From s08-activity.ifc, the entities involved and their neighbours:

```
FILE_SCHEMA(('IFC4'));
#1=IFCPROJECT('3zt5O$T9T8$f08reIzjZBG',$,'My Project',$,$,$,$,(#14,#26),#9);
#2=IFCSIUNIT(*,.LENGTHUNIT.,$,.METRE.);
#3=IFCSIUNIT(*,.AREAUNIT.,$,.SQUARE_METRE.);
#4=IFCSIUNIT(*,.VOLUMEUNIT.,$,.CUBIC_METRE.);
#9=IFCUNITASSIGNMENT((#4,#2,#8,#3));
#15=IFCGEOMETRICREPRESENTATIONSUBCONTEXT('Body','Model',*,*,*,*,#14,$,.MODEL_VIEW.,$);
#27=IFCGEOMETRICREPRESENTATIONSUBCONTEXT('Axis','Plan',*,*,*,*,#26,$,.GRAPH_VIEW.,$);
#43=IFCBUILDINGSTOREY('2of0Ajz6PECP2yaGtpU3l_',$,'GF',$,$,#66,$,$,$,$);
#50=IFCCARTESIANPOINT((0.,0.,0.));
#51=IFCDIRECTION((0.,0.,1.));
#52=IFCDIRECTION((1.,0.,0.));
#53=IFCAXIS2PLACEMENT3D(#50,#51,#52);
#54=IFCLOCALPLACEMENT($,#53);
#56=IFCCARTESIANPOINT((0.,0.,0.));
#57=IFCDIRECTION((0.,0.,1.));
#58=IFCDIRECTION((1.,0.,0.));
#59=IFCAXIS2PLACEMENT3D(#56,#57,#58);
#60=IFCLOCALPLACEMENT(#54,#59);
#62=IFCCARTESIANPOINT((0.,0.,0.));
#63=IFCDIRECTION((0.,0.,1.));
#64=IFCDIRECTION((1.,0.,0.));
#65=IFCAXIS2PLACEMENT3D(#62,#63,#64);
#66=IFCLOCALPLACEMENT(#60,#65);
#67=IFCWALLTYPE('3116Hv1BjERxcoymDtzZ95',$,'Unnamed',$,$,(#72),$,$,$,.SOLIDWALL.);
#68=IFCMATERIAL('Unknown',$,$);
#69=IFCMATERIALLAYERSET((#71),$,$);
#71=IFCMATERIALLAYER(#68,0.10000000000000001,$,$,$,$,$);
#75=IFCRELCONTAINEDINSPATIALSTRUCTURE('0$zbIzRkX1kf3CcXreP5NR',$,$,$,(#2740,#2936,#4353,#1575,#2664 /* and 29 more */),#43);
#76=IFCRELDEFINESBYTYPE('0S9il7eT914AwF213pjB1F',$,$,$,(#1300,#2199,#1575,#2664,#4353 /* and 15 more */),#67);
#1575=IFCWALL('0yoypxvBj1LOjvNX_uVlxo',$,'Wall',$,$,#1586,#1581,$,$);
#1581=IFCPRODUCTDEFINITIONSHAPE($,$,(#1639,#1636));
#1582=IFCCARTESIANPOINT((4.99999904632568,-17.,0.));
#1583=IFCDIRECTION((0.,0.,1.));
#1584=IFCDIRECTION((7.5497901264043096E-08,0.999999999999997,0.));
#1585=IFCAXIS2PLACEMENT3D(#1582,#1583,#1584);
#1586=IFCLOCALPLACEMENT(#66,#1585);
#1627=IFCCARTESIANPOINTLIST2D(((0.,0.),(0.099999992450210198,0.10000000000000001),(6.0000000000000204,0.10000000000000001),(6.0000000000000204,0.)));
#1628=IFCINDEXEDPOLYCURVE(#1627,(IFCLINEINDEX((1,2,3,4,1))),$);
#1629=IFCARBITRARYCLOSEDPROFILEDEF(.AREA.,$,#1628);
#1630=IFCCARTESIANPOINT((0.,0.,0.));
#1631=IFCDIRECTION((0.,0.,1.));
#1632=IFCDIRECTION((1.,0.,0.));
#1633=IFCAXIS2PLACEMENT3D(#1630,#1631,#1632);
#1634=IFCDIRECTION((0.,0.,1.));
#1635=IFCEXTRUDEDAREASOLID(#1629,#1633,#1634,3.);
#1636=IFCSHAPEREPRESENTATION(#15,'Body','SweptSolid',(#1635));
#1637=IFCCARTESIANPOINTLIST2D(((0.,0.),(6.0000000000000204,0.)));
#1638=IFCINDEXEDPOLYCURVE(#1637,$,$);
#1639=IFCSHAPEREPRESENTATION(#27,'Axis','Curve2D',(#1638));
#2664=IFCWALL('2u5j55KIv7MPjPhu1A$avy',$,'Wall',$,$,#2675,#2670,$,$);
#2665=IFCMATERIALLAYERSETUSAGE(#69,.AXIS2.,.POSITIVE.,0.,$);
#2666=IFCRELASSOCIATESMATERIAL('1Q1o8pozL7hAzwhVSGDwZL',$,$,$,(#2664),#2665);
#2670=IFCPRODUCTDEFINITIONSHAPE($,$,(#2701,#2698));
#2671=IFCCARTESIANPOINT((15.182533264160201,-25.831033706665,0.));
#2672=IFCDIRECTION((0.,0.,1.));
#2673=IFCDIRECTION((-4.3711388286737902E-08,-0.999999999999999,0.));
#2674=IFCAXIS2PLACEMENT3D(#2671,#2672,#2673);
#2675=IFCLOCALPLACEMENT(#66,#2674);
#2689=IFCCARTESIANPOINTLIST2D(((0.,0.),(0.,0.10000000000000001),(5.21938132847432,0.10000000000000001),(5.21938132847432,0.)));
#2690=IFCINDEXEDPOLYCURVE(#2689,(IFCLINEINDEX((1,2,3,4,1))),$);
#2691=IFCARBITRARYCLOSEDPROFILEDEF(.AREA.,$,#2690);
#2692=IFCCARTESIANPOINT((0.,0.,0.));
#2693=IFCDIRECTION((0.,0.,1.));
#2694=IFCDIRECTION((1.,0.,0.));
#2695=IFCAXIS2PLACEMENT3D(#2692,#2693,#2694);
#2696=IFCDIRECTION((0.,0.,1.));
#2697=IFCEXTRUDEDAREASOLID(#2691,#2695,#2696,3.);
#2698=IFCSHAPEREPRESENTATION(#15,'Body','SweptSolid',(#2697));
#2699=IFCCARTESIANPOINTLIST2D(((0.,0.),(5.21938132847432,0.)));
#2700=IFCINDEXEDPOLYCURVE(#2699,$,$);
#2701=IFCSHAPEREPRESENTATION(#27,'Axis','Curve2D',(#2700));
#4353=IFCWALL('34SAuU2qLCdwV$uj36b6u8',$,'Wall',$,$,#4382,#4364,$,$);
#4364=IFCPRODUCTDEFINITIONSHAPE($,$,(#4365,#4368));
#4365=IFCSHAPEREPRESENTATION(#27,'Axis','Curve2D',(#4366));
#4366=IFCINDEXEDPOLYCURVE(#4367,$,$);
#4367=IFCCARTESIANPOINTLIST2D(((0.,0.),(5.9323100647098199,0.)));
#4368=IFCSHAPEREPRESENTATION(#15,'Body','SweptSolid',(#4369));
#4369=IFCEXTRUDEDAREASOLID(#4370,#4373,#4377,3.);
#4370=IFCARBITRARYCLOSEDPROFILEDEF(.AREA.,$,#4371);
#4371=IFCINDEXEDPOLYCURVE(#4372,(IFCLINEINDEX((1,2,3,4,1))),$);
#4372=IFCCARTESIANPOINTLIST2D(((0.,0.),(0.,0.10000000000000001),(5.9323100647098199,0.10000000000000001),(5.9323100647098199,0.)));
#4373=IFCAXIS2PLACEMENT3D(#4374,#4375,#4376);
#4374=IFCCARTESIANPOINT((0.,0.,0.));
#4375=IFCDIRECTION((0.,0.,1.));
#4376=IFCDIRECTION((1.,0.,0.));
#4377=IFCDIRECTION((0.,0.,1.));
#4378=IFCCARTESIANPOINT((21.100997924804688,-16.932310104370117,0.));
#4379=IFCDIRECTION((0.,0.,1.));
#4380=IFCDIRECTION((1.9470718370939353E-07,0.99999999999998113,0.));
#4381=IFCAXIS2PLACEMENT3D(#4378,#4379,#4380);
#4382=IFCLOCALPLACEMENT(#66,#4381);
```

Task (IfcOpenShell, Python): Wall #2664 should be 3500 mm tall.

```python
import ifcopenshell
import ifcopenshell.geom
import ifcopenshell.util.representation
import ifcopenshell.util.shape
import ifcopenshell.util.unit

model = ifcopenshell.open("s08-activity.ifc")
unit_scale = ifcopenshell.util.unit.calculate_unit_scale(model)
settings = ifcopenshell.geom.settings()


def volume(element):
    """Net volume in cubic metres, openings subtracted."""
    shape = ifcopenshell.geom.create_shape(settings, element)
    return ifcopenshell.util.shape.get_volume(shape.geometry)


wall = model.by_guid("2u5j55KIv7MPjPhu1A$avy")
before = volume(wall)

body = ifcopenshell.util.representation.get_representation(wall, "Model", "Body")
solid = body.Items[0]
old_height = solid.Depth
solid.Depth = 3.5 / unit_scale
after = volume(wall)

print(f"height {old_height:g} -> {solid.Depth:g}, volume {before:.3f} -> {after:.3f} m3")

model.write("s08-activity_v2.ifc")
```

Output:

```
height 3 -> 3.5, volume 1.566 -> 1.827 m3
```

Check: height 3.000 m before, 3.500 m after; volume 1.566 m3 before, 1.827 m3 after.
